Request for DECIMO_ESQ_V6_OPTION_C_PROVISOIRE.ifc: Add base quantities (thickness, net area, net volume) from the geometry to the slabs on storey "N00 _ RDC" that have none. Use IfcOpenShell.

First a look at what the model holds.

```python
import ifcopenshell
import ifcopenshell.util.element
import ifcopenshell.util.unit

model = ifcopenshell.open("DECIMO_ESQ_V6_OPTION_C_PROVISOIRE.ifc")
print(model.schema)
for unit_type in ("LENGTHUNIT", "AREAUNIT", "VOLUMEUNIT"):
    print(unit_type, ifcopenshell.util.unit.calculate_unit_scale(model, unit_type))
storey = next(s for s in model.by_type("IfcBuildingStorey") if s.Name == "N00 _ RDC")
slabs = [e for e in ifcopenshell.util.element.get_decomposition(storey) if e.is_a("IfcSlab")]
for e in sorted(slabs, key=lambda e: e.id()):
    print(e.id(), e.is_a(), e.Name, list(ifcopenshell.util.element.get_psets(e, qtos_only=True)), sep=" | ")
```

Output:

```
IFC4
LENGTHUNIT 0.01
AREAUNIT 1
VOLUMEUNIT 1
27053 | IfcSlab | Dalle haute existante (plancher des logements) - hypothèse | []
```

```python
import ifcopenshell
import ifcopenshell.api.pset
import ifcopenshell.geom
import ifcopenshell.util.element
import ifcopenshell.util.shape
import ifcopenshell.util.unit

model = ifcopenshell.open("DECIMO_ESQ_V6_OPTION_C_PROVISOIRE.ifc")
unit_scale = ifcopenshell.util.unit.calculate_unit_scale(model)
area_scale = ifcopenshell.util.unit.calculate_unit_scale(model, "AREAUNIT")
volume_scale = ifcopenshell.util.unit.calculate_unit_scale(model, "VOLUMEUNIT")
settings = ifcopenshell.geom.settings()

storey = next(s for s in model.by_type("IfcBuildingStorey") if s.Name == "N00 _ RDC")
slabs = [e for e in ifcopenshell.util.element.get_decomposition(storey) if e.is_a("IfcSlab")]

for e in sorted(slabs, key=lambda e: e.id()):
    if ifcopenshell.util.element.get_psets(e, qtos_only=True, should_inherit=False):
        continue
    # Geometry comes back in metres, in the element's own axes.
    shape = ifcopenshell.geom.create_shape(settings, e)
    values = {
        "Width": ifcopenshell.util.shape.get_z(shape.geometry) / unit_scale,
        "NetArea": ifcopenshell.util.shape.get_footprint_area(shape.geometry) / area_scale,
        "NetVolume": ifcopenshell.util.shape.get_volume(shape.geometry) / volume_scale,
    }
    qto = ifcopenshell.api.pset.add_qto(model, product=e, name="Qto_SlabBaseQuantities")
    ifcopenshell.api.pset.edit_qto(model, qto=qto, properties=values)
    print(e.id(), {k: round(v, 3) for k, v in values.items()})

model.write("DECIMO_ESQ_V6_OPTION_C_PROVISOIRE_rev.ifc")
```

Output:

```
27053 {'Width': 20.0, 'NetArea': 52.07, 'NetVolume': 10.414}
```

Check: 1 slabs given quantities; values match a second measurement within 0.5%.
